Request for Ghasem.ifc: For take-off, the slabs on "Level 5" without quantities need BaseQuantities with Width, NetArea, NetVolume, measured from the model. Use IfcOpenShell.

First a look at what the model holds.

```python
import ifcopenshell
import ifcopenshell.util.element
import ifcopenshell.util.unit

model = ifcopenshell.open("Ghasem.ifc")
print(model.schema)
for unit_type in ("LENGTHUNIT", "AREAUNIT", "VOLUMEUNIT"):
    print(unit_type, ifcopenshell.util.unit.calculate_unit_scale(model, unit_type))
storey = next(s for s in model.by_type("IfcBuildingStorey") if s.Name == "Level 5")
slabs = [e for e in ifcopenshell.util.element.get_decomposition(storey) if e.is_a("IfcSlab")]
for e in sorted(slabs, key=lambda e: e.id()):
    print(e.id(), e.is_a(), e.Name, list(ifcopenshell.util.element.get_psets(e, qtos_only=True)), sep=" | ")
```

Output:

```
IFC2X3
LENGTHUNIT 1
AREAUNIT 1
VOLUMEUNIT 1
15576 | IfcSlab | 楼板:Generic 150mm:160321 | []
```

```python
import ifcopenshell
import ifcopenshell.api.pset
import ifcopenshell.geom
import ifcopenshell.util.element
import ifcopenshell.util.shape
import ifcopenshell.util.unit

model = ifcopenshell.open("Ghasem.ifc")
unit_scale = ifcopenshell.util.unit.calculate_unit_scale(model)
area_scale = ifcopenshell.util.unit.calculate_unit_scale(model, "AREAUNIT")
volume_scale = ifcopenshell.util.unit.calculate_unit_scale(model, "VOLUMEUNIT")
settings = ifcopenshell.geom.settings()

storey = next(s for s in model.by_type("IfcBuildingStorey") if s.Name == "Level 5")
slabs = [e for e in ifcopenshell.util.element.get_decomposition(storey) if e.is_a("IfcSlab")]

for e in sorted(slabs, key=lambda e: e.id()):
    if ifcopenshell.util.element.get_psets(e, qtos_only=True, should_inherit=False):
        continue
    # Geometry comes back in metres, in the element's own axes.
    shape = ifcopenshell.geom.create_shape(settings, e)
    values = {
        "Width": ifcopenshell.util.shape.get_z(shape.geometry) / unit_scale,
        "NetArea": ifcopenshell.util.shape.get_footprint_area(shape.geometry) / area_scale,
        "NetVolume": ifcopenshell.util.shape.get_volume(shape.geometry) / volume_scale,
    }
    qto = ifcopenshell.api.pset.add_qto(model, product=e, name="BaseQuantities")
    ifcopenshell.api.pset.edit_qto(model, qto=qto, properties=values)
    print(e.id(), {k: round(v, 3) for k, v in values.items()})

model.write("Ghasem_edited.ifc")
```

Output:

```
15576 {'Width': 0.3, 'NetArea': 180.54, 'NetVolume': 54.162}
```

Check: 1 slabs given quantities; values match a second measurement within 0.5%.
